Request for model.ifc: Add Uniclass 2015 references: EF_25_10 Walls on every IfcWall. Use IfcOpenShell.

First a look at what the model holds.

```python
import ifcopenshell

model = ifcopenshell.open("model.ifc")
print(model.schema)
print("classifications:", [c.Name for c in model.by_type("IfcClassification")])
for ifc_class in ("IfcDoor", "IfcRoof", "IfcStair", "IfcWall", "IfcWindow"):
    print(ifc_class, len(model.by_type(ifc_class)))
```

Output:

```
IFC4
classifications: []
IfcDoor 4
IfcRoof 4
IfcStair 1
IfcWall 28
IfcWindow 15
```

```python
import ifcopenshell
import ifcopenshell.api.classification

model = ifcopenshell.open("model.ifc")

system = ifcopenshell.api.classification.add_classification(model, classification="Uniclass 2015")

codes = {
    "IfcWall": ("EF_25_10", "Walls"),
}
for ifc_class, (code, name) in codes.items():
    products = model.by_type(ifc_class)
    ifcopenshell.api.classification.add_reference(
        model, products=products, classification=system, identification=code, name=name
    )
    print(code, len(products))

model.write("model-out.ifc")
```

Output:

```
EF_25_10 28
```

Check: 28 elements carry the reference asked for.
